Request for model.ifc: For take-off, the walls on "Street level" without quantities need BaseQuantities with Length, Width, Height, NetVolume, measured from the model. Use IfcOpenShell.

First a look at what the model holds.

```python
import ifcopenshell
import ifcopenshell.util.element
import ifcopenshell.util.unit

model = ifcopenshell.open("model.ifc")
print(model.schema)
for unit_type in ("LENGTHUNIT", "AREAUNIT", "VOLUMEUNIT"):
    print(unit_type, ifcopenshell.util.unit.calculate_unit_scale(model, unit_type))
storey = next(s for s in model.by_type("IfcBuildingStorey") if s.Name == "Street level")
walls = [e for e in ifcopenshell.util.element.get_decomposition(storey) if e.is_a("IfcWall")]
for e in sorted(walls, key=lambda e: e.id()):
    print(e.id(), e.is_a(), e.Name, list(ifcopenshell.util.element.get_psets(e, qtos_only=True)), sep=" | ")
```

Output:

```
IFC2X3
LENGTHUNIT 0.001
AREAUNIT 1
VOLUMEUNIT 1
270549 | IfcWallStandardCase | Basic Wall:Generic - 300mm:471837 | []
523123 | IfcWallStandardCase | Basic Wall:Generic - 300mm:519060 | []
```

```python
import ifcopenshell
import ifcopenshell.api.pset
import ifcopenshell.geom
import ifcopenshell.util.element
import ifcopenshell.util.shape
import ifcopenshell.util.unit

model = ifcopenshell.open("model.ifc")
unit_scale = ifcopenshell.util.unit.calculate_unit_scale(model)
volume_scale = ifcopenshell.util.unit.calculate_unit_scale(model, "VOLUMEUNIT")
settings = ifcopenshell.geom.settings()

storey = next(s for s in model.by_type("IfcBuildingStorey") if s.Name == "Street level")
walls = [e for e in ifcopenshell.util.element.get_decomposition(storey) if e.is_a("IfcWall")]

for e in sorted(walls, key=lambda e: e.id()):
    if ifcopenshell.util.element.get_psets(e, qtos_only=True, should_inherit=False):
        continue
    # Geometry comes back in metres, in the element's own axes.
    shape = ifcopenshell.geom.create_shape(settings, e)
    values = {
        "Length": ifcopenshell.util.shape.get_x(shape.geometry) / unit_scale,
        "Width": ifcopenshell.util.shape.get_y(shape.geometry) / unit_scale,
        "Height": ifcopenshell.util.shape.get_z(shape.geometry) / unit_scale,
        "NetVolume": ifcopenshell.util.shape.get_volume(shape.geometry) / volume_scale,
    }
    qto = ifcopenshell.api.pset.add_qto(model, product=e, name="BaseQuantities")
    ifcopenshell.api.pset.edit_qto(model, qto=qto, properties=values)
    print(e.id(), {k: round(v, 3) for k, v in values.items()})

model.write("model_updated.ifc")
```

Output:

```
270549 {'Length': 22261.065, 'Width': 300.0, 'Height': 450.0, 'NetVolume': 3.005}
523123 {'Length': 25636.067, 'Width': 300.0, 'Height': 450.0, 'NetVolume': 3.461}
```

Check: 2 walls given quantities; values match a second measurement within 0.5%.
